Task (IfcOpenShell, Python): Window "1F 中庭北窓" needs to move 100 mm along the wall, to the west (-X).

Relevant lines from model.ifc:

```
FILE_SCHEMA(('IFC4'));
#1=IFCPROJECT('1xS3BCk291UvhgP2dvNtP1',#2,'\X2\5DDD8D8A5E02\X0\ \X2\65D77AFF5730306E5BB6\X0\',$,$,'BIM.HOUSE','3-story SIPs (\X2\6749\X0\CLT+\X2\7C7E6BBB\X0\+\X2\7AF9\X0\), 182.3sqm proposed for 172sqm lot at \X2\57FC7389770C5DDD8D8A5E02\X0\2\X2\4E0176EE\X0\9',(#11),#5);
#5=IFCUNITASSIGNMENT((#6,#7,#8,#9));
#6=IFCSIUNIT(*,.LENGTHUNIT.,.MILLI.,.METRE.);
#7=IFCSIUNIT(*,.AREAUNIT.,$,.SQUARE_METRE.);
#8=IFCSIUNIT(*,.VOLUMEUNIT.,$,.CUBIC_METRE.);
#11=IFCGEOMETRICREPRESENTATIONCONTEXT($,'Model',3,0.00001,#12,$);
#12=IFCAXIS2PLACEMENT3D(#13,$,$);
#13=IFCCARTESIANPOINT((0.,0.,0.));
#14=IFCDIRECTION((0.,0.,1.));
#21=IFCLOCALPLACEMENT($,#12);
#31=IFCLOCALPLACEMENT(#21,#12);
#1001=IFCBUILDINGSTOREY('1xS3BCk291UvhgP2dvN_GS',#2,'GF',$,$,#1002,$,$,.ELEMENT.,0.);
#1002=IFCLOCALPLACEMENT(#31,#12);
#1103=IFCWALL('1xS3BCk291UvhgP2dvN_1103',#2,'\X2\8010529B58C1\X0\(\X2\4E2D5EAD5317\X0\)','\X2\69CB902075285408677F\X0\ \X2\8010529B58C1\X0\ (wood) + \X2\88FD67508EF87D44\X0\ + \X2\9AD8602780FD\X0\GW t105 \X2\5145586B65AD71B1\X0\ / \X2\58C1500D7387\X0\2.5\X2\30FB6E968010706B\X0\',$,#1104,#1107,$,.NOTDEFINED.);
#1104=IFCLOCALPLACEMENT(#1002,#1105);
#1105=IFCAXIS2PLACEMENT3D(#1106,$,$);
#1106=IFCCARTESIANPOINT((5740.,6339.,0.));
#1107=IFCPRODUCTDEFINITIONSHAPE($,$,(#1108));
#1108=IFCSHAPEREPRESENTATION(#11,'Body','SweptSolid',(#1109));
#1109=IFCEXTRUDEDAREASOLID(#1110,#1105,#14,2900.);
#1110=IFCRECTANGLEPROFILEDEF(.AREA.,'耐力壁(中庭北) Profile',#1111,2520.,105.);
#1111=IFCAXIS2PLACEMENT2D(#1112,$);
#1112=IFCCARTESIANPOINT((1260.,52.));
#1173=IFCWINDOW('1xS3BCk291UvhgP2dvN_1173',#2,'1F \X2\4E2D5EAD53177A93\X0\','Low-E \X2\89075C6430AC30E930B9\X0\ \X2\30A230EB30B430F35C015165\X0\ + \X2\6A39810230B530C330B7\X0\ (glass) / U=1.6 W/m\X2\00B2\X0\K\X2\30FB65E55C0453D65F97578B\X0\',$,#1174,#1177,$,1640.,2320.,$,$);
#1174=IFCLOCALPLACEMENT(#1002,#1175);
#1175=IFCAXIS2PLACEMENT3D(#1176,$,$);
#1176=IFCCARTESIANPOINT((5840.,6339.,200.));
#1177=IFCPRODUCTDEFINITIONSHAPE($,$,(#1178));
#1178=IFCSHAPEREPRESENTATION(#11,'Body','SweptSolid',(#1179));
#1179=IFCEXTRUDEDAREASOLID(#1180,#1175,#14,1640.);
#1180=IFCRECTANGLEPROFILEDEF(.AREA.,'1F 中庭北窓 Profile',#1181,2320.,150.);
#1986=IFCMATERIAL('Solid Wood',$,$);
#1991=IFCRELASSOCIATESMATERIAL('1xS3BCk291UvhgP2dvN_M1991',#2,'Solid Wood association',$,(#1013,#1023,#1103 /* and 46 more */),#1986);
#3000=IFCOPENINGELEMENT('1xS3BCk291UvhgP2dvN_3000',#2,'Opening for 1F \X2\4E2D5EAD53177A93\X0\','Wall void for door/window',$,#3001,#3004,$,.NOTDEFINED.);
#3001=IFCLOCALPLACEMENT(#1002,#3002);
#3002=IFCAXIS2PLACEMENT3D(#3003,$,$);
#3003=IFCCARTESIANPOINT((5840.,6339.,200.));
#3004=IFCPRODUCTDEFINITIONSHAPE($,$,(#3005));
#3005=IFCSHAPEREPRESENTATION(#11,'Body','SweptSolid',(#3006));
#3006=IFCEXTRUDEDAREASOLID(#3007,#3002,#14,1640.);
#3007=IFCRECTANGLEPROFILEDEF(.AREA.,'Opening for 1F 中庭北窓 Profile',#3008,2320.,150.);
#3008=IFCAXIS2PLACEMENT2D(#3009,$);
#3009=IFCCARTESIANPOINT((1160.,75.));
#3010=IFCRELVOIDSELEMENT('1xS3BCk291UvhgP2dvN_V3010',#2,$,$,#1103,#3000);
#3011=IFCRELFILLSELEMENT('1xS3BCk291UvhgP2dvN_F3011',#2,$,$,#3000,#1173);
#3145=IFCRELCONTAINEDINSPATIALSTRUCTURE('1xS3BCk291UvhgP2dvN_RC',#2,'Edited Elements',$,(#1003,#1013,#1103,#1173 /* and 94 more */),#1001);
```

```python
import ifcopenshell
import ifcopenshell.api.geometry
import ifcopenshell.util.placement

model = ifcopenshell.open("model.ifc")

window = model.by_id(1173)
opening = window.FillsVoids[0].RelatingOpeningElement
wall = opening.VoidsElements[0].RelatingBuildingElement

wall_matrix = ifcopenshell.util.placement.get_local_placement(wall.ObjectPlacement)
shift = wall_matrix[:3, 0] * -100.0
before = ifcopenshell.util.placement.get_local_placement(window.ObjectPlacement)[:3, 3].copy()

# The window is not placed relative to its opening, so move both.
for product in (opening, window):
    matrix = ifcopenshell.util.placement.get_local_placement(product.ObjectPlacement)
    matrix[:3, 3] += shift
    ifcopenshell.api.geometry.edit_object_placement(model, product=product, matrix=matrix, is_si=False)

after = ifcopenshell.util.placement.get_local_placement(window.ObjectPlacement)[:3, 3]
print("window moved by", (after - before).round(3) + 0.0)

model.write("model_v2.ifc")
```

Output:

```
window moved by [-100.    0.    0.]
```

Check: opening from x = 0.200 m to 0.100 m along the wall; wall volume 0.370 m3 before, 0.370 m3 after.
